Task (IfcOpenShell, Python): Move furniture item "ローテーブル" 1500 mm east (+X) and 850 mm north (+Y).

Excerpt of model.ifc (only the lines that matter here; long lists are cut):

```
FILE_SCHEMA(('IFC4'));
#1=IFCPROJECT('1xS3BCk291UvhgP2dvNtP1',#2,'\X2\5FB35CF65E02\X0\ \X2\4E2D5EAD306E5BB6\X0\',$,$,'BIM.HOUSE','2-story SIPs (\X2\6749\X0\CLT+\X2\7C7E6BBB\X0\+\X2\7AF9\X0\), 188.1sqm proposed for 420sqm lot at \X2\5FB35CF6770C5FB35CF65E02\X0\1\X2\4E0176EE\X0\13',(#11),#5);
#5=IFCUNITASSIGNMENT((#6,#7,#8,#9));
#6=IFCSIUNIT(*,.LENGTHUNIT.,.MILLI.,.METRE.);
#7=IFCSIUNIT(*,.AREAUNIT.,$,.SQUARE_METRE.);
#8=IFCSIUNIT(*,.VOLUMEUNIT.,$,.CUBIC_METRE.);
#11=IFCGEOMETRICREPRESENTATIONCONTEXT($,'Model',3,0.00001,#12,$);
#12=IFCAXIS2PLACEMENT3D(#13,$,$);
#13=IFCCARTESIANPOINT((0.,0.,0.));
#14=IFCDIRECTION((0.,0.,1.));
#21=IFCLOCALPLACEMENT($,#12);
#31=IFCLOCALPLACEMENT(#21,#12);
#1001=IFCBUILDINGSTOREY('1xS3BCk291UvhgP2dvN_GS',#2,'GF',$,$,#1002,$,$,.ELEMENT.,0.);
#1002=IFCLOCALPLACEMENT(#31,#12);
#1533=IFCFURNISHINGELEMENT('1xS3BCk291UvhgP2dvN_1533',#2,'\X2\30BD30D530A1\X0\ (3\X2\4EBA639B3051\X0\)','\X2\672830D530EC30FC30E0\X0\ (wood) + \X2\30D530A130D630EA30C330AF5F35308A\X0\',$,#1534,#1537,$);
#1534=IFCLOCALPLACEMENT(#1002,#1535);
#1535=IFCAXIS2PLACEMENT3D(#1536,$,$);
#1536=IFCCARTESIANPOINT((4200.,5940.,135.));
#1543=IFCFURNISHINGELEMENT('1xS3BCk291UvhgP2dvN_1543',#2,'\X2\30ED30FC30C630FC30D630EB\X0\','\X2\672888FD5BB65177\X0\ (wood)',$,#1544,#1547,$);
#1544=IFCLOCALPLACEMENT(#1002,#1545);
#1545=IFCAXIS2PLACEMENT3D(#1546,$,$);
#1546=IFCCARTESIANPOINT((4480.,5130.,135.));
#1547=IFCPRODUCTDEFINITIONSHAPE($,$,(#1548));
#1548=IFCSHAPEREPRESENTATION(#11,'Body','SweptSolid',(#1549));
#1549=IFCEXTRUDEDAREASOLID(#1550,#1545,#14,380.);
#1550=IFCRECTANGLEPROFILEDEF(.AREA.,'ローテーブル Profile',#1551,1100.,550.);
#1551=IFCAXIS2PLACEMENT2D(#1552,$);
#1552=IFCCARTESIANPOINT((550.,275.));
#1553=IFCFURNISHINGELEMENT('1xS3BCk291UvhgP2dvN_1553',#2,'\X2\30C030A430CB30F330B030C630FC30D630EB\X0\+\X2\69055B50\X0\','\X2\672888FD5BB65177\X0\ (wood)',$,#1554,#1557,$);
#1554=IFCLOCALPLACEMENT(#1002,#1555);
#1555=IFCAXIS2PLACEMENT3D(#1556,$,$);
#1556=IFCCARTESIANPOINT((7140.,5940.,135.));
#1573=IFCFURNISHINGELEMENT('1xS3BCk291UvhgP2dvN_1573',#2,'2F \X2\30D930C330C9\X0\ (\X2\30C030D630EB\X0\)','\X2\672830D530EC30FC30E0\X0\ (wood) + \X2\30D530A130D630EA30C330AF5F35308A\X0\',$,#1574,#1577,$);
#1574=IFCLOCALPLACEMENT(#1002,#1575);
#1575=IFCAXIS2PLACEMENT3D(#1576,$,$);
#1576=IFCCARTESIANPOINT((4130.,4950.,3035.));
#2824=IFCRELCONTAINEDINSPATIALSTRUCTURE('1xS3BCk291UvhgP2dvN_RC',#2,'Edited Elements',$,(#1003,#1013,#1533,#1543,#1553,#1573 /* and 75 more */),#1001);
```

```python
import ifcopenshell
import ifcopenshell.api.geometry
import ifcopenshell.util.placement
import ifcopenshell.util.unit

model = ifcopenshell.open("model.ifc")
unit_scale = ifcopenshell.util.unit.calculate_unit_scale(model)

item = model.by_guid("1xS3BCk291UvhgP2dvN_1543")
matrix = ifcopenshell.util.placement.get_local_placement(item.ObjectPlacement)
matrix[0, 3] += 1.5 / unit_scale
matrix[1, 3] += 0.85 / unit_scale
ifcopenshell.api.geometry.edit_object_placement(model, product=item, matrix=matrix, is_si=False)

print(ifcopenshell.util.placement.get_local_placement(item.ObjectPlacement).round(3) + 0.0)

model.write("model-out.ifc")
```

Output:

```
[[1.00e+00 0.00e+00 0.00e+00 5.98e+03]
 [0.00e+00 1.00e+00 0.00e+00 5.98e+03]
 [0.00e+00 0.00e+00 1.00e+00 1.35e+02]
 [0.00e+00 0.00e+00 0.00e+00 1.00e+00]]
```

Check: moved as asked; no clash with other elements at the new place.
